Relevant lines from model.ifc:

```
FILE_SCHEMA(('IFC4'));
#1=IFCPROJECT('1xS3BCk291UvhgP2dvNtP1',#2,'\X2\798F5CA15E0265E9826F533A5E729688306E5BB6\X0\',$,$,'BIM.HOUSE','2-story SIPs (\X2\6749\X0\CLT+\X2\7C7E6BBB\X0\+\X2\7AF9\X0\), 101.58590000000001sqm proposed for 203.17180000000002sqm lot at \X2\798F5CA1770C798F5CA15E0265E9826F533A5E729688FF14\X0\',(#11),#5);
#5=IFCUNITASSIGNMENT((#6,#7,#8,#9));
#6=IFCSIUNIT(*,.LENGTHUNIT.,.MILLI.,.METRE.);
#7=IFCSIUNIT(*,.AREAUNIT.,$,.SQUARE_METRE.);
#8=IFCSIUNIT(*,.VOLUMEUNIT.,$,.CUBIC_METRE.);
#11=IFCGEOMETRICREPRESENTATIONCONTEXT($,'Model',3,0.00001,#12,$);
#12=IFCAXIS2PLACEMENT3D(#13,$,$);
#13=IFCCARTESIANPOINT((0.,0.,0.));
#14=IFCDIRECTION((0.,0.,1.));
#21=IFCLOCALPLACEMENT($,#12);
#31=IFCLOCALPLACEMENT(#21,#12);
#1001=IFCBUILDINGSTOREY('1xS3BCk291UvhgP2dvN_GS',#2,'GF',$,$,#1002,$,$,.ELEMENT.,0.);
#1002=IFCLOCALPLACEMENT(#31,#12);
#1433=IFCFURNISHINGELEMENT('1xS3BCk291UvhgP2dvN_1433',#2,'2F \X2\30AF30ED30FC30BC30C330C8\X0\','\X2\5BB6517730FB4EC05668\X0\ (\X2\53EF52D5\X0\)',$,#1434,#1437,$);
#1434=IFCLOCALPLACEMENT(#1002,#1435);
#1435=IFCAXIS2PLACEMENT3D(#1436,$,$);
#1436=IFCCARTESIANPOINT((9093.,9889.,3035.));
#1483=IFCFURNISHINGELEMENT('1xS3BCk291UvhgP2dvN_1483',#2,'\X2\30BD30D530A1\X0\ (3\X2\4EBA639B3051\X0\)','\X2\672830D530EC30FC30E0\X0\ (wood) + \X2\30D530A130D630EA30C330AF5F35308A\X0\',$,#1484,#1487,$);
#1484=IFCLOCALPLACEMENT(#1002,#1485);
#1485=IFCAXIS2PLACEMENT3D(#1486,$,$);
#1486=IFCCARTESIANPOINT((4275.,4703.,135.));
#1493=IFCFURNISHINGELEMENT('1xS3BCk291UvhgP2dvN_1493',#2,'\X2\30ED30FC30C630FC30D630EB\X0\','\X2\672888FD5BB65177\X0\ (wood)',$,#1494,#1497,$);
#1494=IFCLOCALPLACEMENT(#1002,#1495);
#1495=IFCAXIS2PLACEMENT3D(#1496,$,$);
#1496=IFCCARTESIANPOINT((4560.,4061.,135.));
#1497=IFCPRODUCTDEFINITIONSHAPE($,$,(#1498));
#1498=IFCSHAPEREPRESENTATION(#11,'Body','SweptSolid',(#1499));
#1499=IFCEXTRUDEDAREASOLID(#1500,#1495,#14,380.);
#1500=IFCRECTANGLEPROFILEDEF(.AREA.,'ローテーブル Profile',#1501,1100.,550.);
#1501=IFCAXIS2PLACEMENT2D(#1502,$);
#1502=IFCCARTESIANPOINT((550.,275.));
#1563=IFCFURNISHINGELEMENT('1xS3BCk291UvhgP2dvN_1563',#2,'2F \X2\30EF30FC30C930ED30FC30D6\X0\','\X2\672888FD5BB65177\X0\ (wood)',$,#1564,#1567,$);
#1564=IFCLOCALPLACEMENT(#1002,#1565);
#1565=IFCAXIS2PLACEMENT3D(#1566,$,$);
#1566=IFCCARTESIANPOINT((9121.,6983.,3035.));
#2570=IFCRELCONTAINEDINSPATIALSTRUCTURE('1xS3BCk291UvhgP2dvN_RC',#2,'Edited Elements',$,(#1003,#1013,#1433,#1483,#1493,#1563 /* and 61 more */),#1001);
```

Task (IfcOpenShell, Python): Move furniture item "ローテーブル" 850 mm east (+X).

```python
import ifcopenshell
import ifcopenshell.api.geometry
import ifcopenshell.util.placement
import ifcopenshell.util.unit

model = ifcopenshell.open("model.ifc")
unit_scale = ifcopenshell.util.unit.calculate_unit_scale(model)

item = model.by_guid("1xS3BCk291UvhgP2dvN_1493")
matrix = ifcopenshell.util.placement.get_local_placement(item.ObjectPlacement)
matrix[0, 3] += 0.85 / unit_scale
ifcopenshell.api.geometry.edit_object_placement(model, product=item, matrix=matrix, is_si=False)

print(ifcopenshell.util.placement.get_local_placement(item.ObjectPlacement).round(3) + 0.0)

model.write("model_updated.ifc")
```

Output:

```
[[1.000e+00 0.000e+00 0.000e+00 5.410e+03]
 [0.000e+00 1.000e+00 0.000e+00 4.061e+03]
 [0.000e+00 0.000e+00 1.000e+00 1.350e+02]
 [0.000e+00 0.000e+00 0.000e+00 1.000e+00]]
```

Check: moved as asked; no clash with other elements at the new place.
